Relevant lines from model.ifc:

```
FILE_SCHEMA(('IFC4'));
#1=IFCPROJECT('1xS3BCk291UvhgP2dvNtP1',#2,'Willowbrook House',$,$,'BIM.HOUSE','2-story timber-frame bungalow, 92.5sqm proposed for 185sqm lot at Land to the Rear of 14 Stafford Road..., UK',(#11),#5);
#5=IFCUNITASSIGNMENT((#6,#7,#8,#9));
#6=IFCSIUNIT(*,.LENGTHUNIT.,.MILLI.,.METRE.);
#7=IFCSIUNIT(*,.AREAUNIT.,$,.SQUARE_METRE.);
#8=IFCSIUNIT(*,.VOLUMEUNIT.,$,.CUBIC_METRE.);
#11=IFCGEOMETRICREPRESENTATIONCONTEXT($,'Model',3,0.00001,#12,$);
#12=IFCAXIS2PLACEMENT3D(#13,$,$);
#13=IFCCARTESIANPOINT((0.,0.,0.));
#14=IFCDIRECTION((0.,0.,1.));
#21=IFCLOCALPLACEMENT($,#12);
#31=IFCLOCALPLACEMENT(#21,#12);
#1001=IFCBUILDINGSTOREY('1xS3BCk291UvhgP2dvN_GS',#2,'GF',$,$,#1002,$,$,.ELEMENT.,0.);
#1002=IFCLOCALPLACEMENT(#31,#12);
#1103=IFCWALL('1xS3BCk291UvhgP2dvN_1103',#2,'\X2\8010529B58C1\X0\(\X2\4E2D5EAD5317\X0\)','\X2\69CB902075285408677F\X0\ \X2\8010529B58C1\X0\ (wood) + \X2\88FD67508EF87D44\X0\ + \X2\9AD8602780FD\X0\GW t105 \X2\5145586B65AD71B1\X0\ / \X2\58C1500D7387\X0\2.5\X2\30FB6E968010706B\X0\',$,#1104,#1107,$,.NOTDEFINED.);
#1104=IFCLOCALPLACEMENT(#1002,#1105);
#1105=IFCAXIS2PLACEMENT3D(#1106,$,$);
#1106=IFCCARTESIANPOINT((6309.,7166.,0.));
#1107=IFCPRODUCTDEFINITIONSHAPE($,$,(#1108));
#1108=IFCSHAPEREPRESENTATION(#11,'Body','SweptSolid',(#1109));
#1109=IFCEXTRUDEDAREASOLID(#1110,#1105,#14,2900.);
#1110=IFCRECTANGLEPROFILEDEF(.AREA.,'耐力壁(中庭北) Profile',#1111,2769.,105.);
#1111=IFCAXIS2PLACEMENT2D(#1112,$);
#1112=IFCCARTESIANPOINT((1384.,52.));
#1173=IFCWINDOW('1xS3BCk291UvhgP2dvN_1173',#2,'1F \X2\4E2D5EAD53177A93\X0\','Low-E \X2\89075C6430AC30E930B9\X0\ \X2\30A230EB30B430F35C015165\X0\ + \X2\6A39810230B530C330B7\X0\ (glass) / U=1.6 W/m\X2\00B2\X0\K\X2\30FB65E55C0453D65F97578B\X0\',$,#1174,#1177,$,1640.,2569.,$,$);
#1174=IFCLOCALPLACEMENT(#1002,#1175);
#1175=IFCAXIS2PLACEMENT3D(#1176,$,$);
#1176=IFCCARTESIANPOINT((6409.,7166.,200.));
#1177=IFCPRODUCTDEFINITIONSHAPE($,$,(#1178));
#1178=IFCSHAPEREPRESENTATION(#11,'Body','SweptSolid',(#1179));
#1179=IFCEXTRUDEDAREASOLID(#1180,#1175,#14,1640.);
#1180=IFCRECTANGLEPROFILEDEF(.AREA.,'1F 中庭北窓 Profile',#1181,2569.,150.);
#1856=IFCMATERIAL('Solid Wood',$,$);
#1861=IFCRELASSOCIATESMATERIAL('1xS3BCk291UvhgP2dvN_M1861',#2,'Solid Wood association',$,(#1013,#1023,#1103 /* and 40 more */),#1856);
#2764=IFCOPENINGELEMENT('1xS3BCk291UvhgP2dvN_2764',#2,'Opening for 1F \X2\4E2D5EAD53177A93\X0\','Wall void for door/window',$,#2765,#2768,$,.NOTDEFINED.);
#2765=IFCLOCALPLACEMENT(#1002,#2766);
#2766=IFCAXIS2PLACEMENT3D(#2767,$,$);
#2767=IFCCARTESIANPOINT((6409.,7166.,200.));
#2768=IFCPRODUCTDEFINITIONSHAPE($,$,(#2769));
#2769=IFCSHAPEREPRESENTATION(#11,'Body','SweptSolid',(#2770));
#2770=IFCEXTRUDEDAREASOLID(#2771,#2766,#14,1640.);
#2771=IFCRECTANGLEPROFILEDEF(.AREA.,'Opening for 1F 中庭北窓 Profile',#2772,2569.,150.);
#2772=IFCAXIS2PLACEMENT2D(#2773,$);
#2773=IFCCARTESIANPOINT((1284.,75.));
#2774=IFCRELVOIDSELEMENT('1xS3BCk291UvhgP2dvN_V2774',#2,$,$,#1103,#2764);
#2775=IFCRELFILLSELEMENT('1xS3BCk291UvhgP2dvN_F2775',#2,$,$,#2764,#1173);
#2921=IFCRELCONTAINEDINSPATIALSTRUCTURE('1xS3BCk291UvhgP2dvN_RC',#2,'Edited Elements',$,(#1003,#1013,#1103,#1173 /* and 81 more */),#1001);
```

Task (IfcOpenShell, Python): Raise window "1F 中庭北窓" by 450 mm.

```python
import numpy as np
import ifcopenshell
import ifcopenshell.api.geometry
import ifcopenshell.util.placement
import ifcopenshell.util.unit

model = ifcopenshell.open("model.ifc")
unit_scale = ifcopenshell.util.unit.calculate_unit_scale(model)

window = model.by_id(1173)
opening = window.FillsVoids[0].RelatingOpeningElement
dz = 0.45 / unit_scale

shift = np.array([0.0, 0.0, dz])
# The window is not placed relative to its opening, so move both.
for product in (opening, window):
    matrix = ifcopenshell.util.placement.get_local_placement(product.ObjectPlacement)
    matrix[:3, 3] += shift
    ifcopenshell.api.geometry.edit_object_placement(model, product=product, matrix=matrix, is_si=False)

print(f"moved by {dz * unit_scale:+.3f} m")

model.write("model_v2.ifc")
```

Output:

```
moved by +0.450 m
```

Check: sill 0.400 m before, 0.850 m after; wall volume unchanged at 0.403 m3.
